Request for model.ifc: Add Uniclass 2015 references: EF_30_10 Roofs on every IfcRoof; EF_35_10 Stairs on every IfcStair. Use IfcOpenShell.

First a look at what the model holds.

```python
import ifcopenshell

model = ifcopenshell.open("model.ifc")
print(model.schema)
print("classifications:", [c.Name for c in model.by_type("IfcClassification")])
for ifc_class in ("IfcDoor", "IfcRoof", "IfcStair", "IfcWall", "IfcWindow"):
    print(ifc_class, len(model.by_type(ifc_class)))
```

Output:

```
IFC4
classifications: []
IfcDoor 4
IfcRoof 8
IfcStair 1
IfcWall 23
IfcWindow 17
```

```python
import ifcopenshell
import ifcopenshell.api.classification

model = ifcopenshell.open("model.ifc")

system = ifcopenshell.api.classification.add_classification(model, classification="Uniclass 2015")

codes = {
    "IfcRoof": ("EF_30_10", "Roofs"),
    "IfcStair": ("EF_35_10", "Stairs"),
}
for ifc_class, (code, name) in codes.items():
    products = model.by_type(ifc_class)
    ifcopenshell.api.classification.add_reference(
        model, products=products, classification=system, identification=code, name=name
    )
    print(code, len(products))

model.write("model_v2.ifc")
```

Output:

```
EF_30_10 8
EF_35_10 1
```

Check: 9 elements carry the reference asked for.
